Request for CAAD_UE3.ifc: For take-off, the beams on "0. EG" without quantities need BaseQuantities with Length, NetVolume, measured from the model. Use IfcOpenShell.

First a look at what the model holds.

```python
import ifcopenshell
import ifcopenshell.util.element
import ifcopenshell.util.unit

model = ifcopenshell.open("CAAD_UE3.ifc")
print(model.schema)
for unit_type in ("LENGTHUNIT", "AREAUNIT", "VOLUMEUNIT"):
    print(unit_type, ifcopenshell.util.unit.calculate_unit_scale(model, unit_type))
storey = next(s for s in model.by_type("IfcBuildingStorey") if s.Name == "0. EG")
beams = [e for e in ifcopenshell.util.element.get_decomposition(storey) if e.is_a("IfcBeam")]
for e in sorted(beams, key=lambda e: e.id()):
    print(e.id(), e.is_a(), e.Name, list(ifcopenshell.util.element.get_psets(e, qtos_only=True)), sep=" | ")
```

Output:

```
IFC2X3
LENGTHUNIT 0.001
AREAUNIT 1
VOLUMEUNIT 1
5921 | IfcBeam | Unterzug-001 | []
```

```python
import ifcopenshell
import ifcopenshell.api.pset
import ifcopenshell.geom
import ifcopenshell.util.element
import ifcopenshell.util.shape
import ifcopenshell.util.unit

model = ifcopenshell.open("CAAD_UE3.ifc")
unit_scale = ifcopenshell.util.unit.calculate_unit_scale(model)
volume_scale = ifcopenshell.util.unit.calculate_unit_scale(model, "VOLUMEUNIT")
settings = ifcopenshell.geom.settings()

storey = next(s for s in model.by_type("IfcBuildingStorey") if s.Name == "0. EG")
beams = [e for e in ifcopenshell.util.element.get_decomposition(storey) if e.is_a("IfcBeam")]

for e in sorted(beams, key=lambda e: e.id()):
    if ifcopenshell.util.element.get_psets(e, qtos_only=True, should_inherit=False):
        continue
    # Geometry comes back in metres, in the element's own axes.
    shape = ifcopenshell.geom.create_shape(settings, e)
    values = {
        "Length": ifcopenshell.util.shape.get_max_xyz(shape.geometry) / unit_scale,
        "NetVolume": ifcopenshell.util.shape.get_volume(shape.geometry) / volume_scale,
    }
    qto = ifcopenshell.api.pset.add_qto(model, product=e, name="BaseQuantities")
    ifcopenshell.api.pset.edit_qto(model, qto=qto, properties=values)
    print(e.id(), {k: round(v, 3) for k, v in values.items()})

model.write("CAAD_UE3_v2.ifc")
```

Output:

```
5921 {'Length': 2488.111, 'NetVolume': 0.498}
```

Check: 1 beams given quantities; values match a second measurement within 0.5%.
